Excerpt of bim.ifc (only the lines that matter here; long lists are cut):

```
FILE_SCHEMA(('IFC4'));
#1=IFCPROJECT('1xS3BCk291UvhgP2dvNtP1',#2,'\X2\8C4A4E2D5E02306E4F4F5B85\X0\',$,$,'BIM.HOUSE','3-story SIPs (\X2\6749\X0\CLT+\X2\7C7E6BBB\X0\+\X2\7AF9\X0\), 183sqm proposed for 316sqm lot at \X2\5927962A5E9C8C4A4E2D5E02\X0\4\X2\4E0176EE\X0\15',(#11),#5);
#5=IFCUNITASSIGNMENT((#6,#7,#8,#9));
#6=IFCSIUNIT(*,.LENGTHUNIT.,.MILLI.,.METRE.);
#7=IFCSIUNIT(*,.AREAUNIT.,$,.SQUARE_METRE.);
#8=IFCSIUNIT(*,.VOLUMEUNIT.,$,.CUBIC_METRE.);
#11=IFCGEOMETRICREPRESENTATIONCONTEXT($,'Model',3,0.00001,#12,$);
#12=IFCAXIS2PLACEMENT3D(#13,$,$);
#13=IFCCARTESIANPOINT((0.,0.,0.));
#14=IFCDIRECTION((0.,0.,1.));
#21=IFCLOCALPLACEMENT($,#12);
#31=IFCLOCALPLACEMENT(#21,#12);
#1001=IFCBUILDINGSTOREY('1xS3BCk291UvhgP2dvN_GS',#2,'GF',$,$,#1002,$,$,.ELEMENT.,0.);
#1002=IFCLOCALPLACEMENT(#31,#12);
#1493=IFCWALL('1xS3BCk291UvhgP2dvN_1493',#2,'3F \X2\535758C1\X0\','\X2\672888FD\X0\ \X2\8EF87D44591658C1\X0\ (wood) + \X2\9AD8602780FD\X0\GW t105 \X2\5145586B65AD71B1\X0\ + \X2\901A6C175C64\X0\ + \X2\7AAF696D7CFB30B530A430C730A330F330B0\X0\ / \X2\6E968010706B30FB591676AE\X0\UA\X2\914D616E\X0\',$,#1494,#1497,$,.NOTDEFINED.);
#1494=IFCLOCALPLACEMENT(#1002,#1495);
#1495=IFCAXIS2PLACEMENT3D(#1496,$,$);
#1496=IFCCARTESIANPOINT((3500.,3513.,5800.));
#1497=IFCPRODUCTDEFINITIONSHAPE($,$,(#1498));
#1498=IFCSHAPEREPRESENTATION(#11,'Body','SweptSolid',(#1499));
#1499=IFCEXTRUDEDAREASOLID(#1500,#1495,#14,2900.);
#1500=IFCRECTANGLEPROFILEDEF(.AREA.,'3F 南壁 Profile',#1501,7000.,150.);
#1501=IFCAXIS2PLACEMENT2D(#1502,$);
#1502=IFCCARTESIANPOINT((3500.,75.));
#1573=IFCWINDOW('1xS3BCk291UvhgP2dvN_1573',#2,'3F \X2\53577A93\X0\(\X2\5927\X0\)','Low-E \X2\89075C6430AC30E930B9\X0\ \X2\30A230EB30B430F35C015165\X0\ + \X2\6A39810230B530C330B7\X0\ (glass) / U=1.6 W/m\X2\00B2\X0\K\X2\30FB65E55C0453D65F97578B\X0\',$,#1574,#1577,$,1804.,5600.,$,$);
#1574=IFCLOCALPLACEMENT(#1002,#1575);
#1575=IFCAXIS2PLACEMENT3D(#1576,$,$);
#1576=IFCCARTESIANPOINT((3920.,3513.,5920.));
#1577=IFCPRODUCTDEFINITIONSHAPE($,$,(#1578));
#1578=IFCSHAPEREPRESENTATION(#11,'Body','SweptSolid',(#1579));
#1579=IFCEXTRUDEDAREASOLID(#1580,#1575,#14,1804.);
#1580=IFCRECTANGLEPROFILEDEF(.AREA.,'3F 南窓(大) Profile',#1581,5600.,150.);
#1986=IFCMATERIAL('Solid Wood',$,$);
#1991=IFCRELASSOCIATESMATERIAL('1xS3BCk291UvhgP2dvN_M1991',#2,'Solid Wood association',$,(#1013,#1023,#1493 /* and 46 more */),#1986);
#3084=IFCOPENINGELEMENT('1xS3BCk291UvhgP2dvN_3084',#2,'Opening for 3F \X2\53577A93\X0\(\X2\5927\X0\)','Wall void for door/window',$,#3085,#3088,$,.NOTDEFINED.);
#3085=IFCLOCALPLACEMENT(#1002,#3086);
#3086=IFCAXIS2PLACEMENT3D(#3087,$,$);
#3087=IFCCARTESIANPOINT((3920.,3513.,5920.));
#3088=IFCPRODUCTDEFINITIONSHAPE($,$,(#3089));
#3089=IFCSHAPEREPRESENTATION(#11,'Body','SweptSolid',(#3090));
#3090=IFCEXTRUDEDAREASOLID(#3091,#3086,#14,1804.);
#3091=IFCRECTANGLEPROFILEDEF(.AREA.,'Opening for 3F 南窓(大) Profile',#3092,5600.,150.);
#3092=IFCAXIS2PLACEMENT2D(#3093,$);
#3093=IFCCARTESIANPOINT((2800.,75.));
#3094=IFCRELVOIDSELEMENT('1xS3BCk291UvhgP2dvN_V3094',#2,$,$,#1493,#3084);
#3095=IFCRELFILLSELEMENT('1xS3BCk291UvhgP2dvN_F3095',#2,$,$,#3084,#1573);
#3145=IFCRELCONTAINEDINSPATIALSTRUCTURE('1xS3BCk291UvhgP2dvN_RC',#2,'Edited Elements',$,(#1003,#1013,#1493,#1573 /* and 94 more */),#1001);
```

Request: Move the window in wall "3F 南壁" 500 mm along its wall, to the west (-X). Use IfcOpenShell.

```python
import ifcopenshell
import ifcopenshell.api.geometry
import ifcopenshell.util.placement
import ifcopenshell.util.unit

model = ifcopenshell.open("bim.ifc")
unit_scale = ifcopenshell.util.unit.calculate_unit_scale(model)

window = model.by_id(1573)
opening = window.FillsVoids[0].RelatingOpeningElement
wall = opening.VoidsElements[0].RelatingBuildingElement

wall_matrix = ifcopenshell.util.placement.get_local_placement(wall.ObjectPlacement)
shift = wall_matrix[:3, 0] * -0.5 / unit_scale
before = ifcopenshell.util.placement.get_local_placement(window.ObjectPlacement)[:3, 3].copy()

# The window is not placed relative to its opening, so move both.
for product in (opening, window):
    matrix = ifcopenshell.util.placement.get_local_placement(product.ObjectPlacement)
    matrix[:3, 3] += shift
    ifcopenshell.api.geometry.edit_object_placement(model, product=product, matrix=matrix, is_si=False)

after = ifcopenshell.util.placement.get_local_placement(window.ObjectPlacement)[:3, 3]
print("window moved by", (after - before).round(3) + 0.0)

model.write("bim_rev.ifc")
```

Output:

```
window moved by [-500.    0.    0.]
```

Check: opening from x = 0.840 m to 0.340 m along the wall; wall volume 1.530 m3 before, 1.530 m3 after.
